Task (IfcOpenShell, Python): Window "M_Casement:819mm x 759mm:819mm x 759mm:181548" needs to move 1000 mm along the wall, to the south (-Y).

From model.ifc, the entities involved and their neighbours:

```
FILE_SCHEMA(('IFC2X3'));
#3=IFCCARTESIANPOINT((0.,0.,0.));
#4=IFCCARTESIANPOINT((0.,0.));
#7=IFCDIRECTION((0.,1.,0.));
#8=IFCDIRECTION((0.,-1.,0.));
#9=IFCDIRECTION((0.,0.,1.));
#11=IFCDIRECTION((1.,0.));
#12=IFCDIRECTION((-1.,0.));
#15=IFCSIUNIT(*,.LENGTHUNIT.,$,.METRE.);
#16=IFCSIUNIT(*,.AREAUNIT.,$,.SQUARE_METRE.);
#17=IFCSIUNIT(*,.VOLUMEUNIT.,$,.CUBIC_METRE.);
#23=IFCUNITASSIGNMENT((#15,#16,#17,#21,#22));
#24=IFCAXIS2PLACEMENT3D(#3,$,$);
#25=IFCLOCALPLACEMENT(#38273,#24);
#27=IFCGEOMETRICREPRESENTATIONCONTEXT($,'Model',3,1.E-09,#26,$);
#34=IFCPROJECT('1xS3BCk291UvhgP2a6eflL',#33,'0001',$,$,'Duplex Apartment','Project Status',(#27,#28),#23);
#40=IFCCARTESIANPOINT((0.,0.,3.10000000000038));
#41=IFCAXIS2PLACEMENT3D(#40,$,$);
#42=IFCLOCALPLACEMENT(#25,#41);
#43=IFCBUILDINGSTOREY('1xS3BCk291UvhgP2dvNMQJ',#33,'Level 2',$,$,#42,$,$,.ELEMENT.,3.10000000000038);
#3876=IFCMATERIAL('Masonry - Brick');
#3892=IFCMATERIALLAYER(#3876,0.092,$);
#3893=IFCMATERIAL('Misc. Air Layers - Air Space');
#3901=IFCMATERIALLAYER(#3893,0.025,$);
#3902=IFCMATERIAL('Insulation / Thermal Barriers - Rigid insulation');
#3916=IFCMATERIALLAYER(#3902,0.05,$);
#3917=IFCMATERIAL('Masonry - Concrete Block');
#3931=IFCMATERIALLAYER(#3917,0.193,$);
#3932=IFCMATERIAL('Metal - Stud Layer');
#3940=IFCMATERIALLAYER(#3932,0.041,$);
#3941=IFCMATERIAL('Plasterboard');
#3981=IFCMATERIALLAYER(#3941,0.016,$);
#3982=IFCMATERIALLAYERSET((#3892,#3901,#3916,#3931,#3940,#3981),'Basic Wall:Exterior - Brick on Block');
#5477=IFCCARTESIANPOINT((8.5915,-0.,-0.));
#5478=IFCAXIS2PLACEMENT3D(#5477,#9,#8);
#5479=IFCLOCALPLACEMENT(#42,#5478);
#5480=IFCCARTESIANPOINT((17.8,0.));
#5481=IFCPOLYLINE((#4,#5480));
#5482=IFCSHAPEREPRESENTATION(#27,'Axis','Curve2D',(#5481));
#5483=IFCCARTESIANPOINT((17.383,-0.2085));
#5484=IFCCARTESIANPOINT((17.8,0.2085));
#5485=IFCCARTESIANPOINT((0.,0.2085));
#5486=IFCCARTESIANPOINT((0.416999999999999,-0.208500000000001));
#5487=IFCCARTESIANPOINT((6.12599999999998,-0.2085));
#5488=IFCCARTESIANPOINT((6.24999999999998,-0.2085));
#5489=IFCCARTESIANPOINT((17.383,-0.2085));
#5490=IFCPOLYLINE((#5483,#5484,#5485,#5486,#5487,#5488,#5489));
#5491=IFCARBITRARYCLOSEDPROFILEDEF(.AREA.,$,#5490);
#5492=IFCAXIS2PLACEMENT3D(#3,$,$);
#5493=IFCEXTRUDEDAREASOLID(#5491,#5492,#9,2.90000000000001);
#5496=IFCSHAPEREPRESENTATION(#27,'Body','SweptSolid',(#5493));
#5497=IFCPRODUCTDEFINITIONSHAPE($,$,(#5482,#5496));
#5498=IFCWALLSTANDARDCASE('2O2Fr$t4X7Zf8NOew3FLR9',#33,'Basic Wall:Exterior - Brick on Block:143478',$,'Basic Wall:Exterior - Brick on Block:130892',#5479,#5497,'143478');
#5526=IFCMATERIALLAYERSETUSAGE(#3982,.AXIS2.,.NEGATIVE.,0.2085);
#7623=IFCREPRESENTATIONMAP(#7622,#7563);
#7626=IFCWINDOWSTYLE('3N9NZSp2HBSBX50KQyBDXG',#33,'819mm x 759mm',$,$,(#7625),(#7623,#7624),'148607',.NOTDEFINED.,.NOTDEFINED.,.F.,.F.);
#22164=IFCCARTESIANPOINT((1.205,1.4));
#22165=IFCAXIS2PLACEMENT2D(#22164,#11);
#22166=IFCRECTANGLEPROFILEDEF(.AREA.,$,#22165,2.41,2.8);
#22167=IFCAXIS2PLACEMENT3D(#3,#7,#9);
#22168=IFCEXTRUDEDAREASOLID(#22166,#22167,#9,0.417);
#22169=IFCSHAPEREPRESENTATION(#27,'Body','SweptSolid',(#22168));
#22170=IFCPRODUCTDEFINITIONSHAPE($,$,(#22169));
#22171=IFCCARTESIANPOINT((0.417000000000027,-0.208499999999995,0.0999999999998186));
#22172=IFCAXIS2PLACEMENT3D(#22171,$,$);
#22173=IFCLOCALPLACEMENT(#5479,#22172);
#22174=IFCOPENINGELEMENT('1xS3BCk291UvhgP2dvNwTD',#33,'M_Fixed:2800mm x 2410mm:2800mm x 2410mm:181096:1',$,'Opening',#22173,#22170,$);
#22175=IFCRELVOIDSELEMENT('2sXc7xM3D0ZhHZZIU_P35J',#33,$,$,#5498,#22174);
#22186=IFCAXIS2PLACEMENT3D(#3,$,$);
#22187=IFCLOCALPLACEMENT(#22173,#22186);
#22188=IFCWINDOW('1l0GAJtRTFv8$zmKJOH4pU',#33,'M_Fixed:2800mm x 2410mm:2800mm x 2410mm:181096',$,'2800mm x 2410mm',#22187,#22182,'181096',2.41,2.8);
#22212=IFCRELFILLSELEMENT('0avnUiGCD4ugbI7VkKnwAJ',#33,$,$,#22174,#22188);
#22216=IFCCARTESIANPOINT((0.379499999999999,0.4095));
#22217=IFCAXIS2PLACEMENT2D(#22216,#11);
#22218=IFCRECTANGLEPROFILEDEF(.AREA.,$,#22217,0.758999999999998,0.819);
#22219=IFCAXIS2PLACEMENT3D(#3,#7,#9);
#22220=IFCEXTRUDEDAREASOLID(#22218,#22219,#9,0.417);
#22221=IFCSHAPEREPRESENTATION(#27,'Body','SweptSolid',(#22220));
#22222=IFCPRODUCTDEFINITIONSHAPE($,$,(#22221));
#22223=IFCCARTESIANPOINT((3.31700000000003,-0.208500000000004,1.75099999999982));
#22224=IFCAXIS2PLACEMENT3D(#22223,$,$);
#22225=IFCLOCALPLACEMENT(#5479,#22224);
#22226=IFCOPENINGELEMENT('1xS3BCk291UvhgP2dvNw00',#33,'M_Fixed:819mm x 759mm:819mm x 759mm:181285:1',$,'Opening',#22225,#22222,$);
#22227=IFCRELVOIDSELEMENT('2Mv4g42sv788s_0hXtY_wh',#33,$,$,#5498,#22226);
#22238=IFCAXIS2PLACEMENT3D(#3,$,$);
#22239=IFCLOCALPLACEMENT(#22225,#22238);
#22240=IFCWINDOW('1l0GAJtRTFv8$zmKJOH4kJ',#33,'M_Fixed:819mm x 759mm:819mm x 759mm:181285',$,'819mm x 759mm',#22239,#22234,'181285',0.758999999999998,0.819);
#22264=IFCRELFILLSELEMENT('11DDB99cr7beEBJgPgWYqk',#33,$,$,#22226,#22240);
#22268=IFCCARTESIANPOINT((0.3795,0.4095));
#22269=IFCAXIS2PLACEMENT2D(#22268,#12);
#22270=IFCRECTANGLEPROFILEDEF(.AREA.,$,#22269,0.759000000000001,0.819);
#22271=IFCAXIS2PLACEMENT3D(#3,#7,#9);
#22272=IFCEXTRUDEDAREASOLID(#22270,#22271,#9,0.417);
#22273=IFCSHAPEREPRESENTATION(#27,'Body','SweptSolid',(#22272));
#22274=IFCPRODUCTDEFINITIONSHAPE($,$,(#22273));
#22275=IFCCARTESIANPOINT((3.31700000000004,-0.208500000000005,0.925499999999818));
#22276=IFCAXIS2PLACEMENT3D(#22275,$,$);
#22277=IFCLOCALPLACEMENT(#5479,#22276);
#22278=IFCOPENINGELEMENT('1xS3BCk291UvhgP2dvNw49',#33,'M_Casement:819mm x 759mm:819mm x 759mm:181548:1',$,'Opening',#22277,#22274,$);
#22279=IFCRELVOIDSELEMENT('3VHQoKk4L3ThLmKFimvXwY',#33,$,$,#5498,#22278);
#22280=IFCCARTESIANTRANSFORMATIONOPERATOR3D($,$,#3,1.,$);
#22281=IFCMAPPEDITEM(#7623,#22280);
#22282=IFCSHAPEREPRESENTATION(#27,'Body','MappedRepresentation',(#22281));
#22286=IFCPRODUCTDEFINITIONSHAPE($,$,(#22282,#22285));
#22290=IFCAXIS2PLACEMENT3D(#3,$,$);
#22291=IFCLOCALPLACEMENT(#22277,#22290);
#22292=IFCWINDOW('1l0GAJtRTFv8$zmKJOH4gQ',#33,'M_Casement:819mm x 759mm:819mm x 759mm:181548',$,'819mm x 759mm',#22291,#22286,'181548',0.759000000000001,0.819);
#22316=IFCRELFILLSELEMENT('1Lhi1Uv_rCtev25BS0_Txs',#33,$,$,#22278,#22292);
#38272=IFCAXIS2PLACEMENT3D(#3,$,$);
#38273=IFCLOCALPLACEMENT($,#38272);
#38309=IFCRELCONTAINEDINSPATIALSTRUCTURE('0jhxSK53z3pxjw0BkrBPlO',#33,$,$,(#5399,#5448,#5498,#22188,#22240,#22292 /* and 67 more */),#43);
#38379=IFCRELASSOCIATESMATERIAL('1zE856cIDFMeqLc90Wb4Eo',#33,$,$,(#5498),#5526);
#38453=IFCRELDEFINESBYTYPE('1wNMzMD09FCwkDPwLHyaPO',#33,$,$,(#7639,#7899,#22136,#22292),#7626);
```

```python
import ifcopenshell
import ifcopenshell.api.geometry
import ifcopenshell.util.placement
import ifcopenshell.util.unit

model = ifcopenshell.open("model.ifc")
unit_scale = ifcopenshell.util.unit.calculate_unit_scale(model)

window = model.by_id(22292)
opening = window.FillsVoids[0].RelatingOpeningElement
wall = opening.VoidsElements[0].RelatingBuildingElement

wall_matrix = ifcopenshell.util.placement.get_local_placement(wall.ObjectPlacement)
shift = wall_matrix[:3, 0] * 1 / unit_scale
before = ifcopenshell.util.placement.get_local_placement(window.ObjectPlacement)[:3, 3].copy()

# The window is placed relative to its opening, so it follows when the opening moves.
matrix = ifcopenshell.util.placement.get_local_placement(opening.ObjectPlacement)
matrix[:3, 3] += shift
ifcopenshell.api.geometry.edit_object_placement(
    model, product=opening, matrix=matrix, is_si=False, should_transform_children=True
)

after = ifcopenshell.util.placement.get_local_placement(window.ObjectPlacement)[:3, 3]
print("window moved by", (after - before).round(3) + 0.0)

model.write("model-out.ifc")
```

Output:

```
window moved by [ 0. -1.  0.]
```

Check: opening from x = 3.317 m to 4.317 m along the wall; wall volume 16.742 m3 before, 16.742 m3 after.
